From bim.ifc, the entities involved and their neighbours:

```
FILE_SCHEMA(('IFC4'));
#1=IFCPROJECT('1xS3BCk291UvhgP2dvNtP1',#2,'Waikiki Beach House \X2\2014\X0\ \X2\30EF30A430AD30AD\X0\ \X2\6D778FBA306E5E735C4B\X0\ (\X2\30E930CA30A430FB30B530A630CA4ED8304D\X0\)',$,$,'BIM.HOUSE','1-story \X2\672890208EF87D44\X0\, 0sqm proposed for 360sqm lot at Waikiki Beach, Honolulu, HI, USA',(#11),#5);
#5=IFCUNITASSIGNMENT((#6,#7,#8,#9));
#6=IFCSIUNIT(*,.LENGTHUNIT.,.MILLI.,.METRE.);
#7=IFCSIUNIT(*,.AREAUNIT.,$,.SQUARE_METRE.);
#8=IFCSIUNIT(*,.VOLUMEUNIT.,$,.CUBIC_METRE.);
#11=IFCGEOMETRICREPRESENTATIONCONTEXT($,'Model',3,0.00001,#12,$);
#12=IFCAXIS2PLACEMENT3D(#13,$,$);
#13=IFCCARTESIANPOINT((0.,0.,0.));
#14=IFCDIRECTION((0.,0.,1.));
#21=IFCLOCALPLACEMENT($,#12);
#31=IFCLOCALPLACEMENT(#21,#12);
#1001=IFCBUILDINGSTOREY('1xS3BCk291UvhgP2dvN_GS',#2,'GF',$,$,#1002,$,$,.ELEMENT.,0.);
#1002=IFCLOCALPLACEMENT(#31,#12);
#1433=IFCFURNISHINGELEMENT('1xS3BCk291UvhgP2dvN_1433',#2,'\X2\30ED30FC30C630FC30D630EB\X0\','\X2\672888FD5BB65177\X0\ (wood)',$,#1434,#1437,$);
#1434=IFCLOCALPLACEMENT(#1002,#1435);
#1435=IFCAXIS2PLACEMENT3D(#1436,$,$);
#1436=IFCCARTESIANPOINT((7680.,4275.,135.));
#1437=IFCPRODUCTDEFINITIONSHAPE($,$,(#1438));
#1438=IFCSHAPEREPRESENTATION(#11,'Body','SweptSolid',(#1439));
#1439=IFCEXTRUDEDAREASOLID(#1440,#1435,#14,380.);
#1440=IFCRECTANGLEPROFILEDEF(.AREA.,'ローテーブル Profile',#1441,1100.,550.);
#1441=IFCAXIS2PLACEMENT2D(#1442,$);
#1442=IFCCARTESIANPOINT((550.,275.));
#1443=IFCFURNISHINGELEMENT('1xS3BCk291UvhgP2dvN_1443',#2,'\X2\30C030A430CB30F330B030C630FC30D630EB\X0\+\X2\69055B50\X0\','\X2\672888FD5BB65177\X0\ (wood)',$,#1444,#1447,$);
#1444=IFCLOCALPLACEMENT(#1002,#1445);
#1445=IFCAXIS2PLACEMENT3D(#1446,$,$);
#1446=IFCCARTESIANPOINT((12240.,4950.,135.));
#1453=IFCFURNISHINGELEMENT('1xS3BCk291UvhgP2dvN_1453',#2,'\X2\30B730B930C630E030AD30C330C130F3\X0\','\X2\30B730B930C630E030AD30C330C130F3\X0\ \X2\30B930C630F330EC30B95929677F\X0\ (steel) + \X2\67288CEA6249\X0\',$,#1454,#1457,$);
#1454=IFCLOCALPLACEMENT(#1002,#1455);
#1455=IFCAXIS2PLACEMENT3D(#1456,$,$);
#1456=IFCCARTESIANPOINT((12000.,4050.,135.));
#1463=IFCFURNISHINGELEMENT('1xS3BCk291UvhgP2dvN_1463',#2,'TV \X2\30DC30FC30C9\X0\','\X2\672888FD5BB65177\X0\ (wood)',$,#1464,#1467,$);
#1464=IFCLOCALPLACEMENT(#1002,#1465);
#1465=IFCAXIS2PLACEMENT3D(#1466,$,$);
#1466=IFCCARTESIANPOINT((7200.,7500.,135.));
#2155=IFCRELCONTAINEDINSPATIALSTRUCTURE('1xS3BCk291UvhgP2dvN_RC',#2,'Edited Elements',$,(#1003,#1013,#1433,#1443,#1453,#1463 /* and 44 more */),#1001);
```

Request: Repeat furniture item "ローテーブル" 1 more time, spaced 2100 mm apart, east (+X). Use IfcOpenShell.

```python
import numpy as np
import ifcopenshell
import ifcopenshell.api.geometry
import ifcopenshell.api.root
import ifcopenshell.util.element
import ifcopenshell.util.placement
import ifcopenshell.util.unit

model = ifcopenshell.open("bim.ifc")
unit_scale = ifcopenshell.util.unit.calculate_unit_scale(model)


def reuse_history(source, copy):
    """copy_class also copies each property set's owner history, people and application; keep the originals."""
    for rel in copy.IsDefinedBy:
        if rel.is_a("IfcRelDefinesByProperties") and (history := rel.RelatingPropertyDefinition.OwnerHistory):
            rel.RelatingPropertyDefinition.OwnerHistory = source.OwnerHistory
            ifcopenshell.util.element.remove_deep2(model, history)


source = model.by_guid("1xS3BCk291UvhgP2dvN_1433")
base = ifcopenshell.util.placement.get_local_placement(source.ObjectPlacement)
step = np.array([1.0, 0.0, 0.0]) * 2.1 / unit_scale

for i in range(1, 2):
    copy = ifcopenshell.api.root.copy_class(model, product=source)
    copy.Representation = ifcopenshell.util.element.copy_deep(
        model, source.Representation, exclude=["IfcGeometricRepresentationContext", "IfcRepresentationMap"]
    )
    reuse_history(source, copy)
    matrix = base.copy()
    matrix[:3, 3] += i * step
    print("added at", matrix[:3, 3].round(3) + 0.0)
    ifcopenshell.api.geometry.edit_object_placement(model, product=copy, matrix=matrix, is_si=False)

model.write("bim-out.ifc")
```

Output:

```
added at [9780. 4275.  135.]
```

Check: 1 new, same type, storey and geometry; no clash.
